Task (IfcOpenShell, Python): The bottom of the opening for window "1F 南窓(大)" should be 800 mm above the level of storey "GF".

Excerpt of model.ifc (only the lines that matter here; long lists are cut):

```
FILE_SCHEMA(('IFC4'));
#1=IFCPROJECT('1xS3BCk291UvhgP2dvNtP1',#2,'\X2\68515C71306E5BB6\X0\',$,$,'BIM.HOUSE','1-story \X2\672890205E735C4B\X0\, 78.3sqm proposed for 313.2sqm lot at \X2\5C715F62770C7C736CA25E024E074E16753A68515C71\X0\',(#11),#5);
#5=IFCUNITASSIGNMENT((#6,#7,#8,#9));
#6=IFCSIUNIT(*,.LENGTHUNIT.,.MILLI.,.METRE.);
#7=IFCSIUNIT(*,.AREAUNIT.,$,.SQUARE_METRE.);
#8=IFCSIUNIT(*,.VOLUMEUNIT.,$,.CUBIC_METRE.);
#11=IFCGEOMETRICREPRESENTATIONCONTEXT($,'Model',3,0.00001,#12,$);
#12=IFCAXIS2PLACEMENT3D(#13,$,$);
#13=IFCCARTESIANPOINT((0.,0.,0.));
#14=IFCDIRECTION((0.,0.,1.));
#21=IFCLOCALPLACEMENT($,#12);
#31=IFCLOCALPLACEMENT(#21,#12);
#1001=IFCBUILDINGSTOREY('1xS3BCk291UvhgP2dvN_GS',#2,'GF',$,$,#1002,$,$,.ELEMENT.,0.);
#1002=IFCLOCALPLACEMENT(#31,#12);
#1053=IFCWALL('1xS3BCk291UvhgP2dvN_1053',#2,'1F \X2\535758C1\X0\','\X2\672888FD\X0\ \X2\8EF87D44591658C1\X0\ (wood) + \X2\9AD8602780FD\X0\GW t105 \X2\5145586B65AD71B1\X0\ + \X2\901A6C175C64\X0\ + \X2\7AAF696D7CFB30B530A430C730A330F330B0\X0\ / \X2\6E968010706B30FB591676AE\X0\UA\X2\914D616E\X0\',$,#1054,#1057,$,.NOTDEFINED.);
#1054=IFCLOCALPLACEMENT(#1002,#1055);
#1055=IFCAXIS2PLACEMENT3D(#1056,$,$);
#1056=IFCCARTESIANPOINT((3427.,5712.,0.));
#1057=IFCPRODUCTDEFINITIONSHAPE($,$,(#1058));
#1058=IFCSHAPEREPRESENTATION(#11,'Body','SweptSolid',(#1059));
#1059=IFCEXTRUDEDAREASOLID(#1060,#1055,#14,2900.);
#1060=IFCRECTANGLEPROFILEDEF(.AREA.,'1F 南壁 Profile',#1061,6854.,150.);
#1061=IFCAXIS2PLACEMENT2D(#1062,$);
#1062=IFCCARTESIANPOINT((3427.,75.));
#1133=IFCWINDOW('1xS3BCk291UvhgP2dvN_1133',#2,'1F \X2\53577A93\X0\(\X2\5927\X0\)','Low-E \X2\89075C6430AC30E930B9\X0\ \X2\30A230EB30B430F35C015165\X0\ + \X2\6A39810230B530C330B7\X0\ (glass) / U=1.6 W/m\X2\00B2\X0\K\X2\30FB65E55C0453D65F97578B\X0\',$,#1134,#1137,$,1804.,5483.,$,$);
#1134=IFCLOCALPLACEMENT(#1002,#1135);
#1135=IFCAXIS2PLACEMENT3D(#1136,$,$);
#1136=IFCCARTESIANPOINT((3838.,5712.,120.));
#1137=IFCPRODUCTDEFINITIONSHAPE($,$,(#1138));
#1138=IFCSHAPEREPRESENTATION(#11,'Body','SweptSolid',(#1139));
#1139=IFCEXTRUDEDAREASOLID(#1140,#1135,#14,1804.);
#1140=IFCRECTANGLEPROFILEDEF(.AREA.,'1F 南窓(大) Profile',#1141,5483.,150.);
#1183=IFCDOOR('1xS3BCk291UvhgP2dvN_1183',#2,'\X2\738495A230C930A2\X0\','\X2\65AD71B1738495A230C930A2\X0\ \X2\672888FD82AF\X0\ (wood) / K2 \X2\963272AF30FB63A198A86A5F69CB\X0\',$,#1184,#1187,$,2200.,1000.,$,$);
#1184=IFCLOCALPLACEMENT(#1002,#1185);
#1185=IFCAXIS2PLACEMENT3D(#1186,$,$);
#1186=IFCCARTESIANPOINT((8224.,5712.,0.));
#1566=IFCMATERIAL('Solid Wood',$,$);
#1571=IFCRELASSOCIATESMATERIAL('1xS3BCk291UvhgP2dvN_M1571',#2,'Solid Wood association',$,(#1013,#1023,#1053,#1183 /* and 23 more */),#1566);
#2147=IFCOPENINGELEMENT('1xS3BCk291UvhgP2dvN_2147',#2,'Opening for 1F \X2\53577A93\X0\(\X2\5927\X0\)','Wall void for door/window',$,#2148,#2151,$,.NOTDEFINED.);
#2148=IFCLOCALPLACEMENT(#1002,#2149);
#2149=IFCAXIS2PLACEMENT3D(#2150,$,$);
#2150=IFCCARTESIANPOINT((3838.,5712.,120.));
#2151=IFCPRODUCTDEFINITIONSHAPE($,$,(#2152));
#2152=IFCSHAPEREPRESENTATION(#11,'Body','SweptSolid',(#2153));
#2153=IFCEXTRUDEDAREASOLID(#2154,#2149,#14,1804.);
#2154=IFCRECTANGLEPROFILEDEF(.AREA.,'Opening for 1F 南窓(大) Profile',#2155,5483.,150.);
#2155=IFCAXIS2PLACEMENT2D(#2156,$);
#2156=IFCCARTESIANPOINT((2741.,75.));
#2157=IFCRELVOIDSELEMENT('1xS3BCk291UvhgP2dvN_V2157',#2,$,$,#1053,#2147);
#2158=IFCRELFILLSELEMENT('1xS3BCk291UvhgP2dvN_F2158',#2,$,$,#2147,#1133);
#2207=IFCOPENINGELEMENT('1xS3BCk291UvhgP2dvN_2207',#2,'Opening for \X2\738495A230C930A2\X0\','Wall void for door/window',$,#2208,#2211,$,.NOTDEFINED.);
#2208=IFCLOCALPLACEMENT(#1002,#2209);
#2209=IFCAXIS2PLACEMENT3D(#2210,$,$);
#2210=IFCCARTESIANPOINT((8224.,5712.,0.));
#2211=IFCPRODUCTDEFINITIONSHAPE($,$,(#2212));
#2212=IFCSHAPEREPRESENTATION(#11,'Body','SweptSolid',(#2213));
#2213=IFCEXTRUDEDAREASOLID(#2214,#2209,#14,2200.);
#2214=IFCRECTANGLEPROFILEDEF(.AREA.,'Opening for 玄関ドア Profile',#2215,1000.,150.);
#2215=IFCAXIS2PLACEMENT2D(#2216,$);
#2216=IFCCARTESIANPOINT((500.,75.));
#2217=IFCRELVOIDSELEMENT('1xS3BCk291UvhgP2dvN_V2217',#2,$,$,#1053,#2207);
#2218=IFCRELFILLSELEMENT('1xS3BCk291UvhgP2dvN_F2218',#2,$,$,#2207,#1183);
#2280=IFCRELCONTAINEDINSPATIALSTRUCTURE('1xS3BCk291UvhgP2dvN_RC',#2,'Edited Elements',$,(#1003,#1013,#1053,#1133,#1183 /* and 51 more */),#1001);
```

```python
import numpy as np
import ifcopenshell
import ifcopenshell.api.geometry
import ifcopenshell.geom
import ifcopenshell.util.element
import ifcopenshell.util.placement
import ifcopenshell.util.shape
import ifcopenshell.util.unit

model = ifcopenshell.open("model.ifc")
unit_scale = ifcopenshell.util.unit.calculate_unit_scale(model)

window = model.by_id(1133)
opening = window.FillsVoids[0].RelatingOpeningElement
storey = ifcopenshell.util.element.get_container(window, ifc_class="IfcBuildingStorey")
level = ifcopenshell.util.placement.get_local_placement(storey.ObjectPlacement)[2, 3]

# The opening's origin need not be at the sill, so measure its lowest point.
shape = ifcopenshell.geom.create_shape(ifcopenshell.geom.settings(), opening)
bottom = ifcopenshell.util.shape.get_shape_bottom_elevation(shape, shape.geometry) / unit_scale
dz = level + 0.8 / unit_scale - bottom

shift = np.array([0.0, 0.0, dz])
# The window is not placed relative to its opening, so move both.
for product in (opening, window):
    matrix = ifcopenshell.util.placement.get_local_placement(product.ObjectPlacement)
    matrix[:3, 3] += shift
    ifcopenshell.api.geometry.edit_object_placement(model, product=product, matrix=matrix, is_si=False)

print(f"moved by {dz * unit_scale:+.3f} m")

model.write("model_edited.ifc")
```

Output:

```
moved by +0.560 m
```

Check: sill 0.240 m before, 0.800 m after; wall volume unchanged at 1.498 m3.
